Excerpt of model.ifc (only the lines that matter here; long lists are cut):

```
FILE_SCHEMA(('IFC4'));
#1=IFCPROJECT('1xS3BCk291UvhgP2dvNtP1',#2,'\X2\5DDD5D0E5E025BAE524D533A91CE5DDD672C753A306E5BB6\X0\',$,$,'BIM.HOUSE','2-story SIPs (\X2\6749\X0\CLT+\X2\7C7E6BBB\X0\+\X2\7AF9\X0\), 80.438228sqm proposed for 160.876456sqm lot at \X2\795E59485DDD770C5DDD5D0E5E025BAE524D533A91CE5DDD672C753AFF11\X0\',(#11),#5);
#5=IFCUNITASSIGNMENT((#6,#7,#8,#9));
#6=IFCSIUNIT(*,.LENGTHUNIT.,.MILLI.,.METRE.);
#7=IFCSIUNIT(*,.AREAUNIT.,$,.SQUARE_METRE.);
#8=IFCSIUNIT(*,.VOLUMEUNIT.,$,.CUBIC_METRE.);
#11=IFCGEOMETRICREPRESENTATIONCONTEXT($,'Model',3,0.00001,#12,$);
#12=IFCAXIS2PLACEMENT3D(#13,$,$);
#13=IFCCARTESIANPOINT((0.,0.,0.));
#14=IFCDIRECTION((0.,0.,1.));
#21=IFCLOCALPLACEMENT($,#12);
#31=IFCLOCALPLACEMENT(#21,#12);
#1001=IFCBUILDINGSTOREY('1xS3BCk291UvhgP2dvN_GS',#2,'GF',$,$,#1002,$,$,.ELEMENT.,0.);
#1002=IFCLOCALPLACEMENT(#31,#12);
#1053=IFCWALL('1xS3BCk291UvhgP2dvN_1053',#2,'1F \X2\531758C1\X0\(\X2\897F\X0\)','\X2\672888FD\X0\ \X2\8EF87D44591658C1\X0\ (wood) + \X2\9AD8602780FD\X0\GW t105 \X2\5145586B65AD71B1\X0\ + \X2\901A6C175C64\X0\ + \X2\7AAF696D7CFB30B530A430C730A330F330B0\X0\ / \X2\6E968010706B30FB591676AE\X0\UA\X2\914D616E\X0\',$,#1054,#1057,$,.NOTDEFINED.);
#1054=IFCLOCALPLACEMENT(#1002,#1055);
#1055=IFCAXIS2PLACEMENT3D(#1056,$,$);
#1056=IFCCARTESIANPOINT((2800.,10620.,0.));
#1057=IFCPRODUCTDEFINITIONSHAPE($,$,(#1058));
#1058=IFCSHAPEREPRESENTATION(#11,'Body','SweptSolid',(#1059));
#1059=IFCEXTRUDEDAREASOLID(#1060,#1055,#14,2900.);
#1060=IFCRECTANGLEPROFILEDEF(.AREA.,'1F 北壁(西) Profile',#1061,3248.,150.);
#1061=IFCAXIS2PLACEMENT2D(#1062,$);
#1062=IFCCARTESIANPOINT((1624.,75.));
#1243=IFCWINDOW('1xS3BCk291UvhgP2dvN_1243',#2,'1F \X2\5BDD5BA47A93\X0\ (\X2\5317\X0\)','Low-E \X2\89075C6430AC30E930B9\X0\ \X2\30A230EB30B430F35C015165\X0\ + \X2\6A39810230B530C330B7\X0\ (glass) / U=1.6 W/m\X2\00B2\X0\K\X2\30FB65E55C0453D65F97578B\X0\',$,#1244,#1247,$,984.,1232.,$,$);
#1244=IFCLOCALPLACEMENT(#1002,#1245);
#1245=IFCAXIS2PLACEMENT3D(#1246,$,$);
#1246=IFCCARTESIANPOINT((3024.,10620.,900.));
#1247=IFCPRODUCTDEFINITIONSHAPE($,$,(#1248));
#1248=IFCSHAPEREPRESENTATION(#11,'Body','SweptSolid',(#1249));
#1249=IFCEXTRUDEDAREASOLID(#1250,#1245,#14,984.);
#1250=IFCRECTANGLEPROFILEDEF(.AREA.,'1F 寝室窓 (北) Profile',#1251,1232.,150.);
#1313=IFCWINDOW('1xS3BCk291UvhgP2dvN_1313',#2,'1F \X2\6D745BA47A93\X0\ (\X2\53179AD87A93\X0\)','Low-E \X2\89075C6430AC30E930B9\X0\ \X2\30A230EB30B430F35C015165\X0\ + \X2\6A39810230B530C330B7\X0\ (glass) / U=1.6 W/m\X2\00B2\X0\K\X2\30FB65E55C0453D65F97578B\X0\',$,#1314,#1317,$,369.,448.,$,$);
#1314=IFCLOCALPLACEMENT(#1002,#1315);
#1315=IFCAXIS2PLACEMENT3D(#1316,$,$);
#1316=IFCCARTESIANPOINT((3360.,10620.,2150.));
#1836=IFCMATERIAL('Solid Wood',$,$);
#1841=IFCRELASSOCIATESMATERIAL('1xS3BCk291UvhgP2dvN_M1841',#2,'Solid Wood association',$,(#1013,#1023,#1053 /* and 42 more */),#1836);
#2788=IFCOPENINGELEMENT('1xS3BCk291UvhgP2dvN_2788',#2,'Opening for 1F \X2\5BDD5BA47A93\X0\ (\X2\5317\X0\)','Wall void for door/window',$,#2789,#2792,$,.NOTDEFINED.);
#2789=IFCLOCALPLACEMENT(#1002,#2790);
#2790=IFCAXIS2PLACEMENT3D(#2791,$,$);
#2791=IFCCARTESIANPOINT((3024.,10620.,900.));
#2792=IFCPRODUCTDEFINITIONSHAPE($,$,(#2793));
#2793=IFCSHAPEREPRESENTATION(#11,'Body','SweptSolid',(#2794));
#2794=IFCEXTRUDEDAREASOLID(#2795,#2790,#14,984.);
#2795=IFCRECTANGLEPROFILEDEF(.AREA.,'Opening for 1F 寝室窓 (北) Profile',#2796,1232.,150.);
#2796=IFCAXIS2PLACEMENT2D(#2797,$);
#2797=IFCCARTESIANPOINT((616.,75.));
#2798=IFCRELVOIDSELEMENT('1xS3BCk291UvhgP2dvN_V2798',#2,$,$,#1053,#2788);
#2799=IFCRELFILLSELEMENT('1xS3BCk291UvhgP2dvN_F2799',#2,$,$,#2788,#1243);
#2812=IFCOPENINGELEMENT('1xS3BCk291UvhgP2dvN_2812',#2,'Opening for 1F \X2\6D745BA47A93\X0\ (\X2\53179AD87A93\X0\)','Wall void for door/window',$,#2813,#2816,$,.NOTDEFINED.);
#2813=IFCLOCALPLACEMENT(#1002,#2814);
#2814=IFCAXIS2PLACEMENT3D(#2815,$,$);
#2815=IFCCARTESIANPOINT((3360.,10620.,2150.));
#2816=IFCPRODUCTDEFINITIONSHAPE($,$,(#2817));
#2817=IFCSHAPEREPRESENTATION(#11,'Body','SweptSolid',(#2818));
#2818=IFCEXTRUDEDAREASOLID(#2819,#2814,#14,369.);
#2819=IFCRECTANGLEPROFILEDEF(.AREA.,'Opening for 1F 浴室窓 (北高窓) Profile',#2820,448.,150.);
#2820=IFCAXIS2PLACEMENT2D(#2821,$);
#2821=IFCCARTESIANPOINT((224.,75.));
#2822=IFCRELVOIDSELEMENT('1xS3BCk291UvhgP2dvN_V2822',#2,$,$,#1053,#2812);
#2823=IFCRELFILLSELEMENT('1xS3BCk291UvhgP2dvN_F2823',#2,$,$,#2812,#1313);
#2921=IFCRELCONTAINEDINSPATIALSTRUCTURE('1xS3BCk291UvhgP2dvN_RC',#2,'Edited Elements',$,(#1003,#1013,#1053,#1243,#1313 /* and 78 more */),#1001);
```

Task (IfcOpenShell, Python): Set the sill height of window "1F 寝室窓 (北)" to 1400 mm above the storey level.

```python
import numpy as np
import ifcopenshell
import ifcopenshell.api.geometry
import ifcopenshell.geom
import ifcopenshell.util.element
import ifcopenshell.util.placement
import ifcopenshell.util.shape
import ifcopenshell.util.unit

model = ifcopenshell.open("model.ifc")
unit_scale = ifcopenshell.util.unit.calculate_unit_scale(model)

window = model.by_id(1243)
opening = window.FillsVoids[0].RelatingOpeningElement
storey = ifcopenshell.util.element.get_container(window, ifc_class="IfcBuildingStorey")
level = ifcopenshell.util.placement.get_local_placement(storey.ObjectPlacement)[2, 3]

# The opening's origin need not be at the sill, so measure its lowest point.
shape = ifcopenshell.geom.create_shape(ifcopenshell.geom.settings(), opening)
bottom = ifcopenshell.util.shape.get_shape_bottom_elevation(shape, shape.geometry) / unit_scale
dz = level + 1400.0 - bottom

shift = np.array([0.0, 0.0, dz])
# The window is not placed relative to its opening, so move both.
for product in (opening, window):
    matrix = ifcopenshell.util.placement.get_local_placement(product.ObjectPlacement)
    matrix[:3, 3] += shift
    ifcopenshell.api.geometry.edit_object_placement(model, product=product, matrix=matrix, is_si=False)

print(f"moved by {dz * unit_scale:+.3f} m")

model.write("model-out.ifc")
```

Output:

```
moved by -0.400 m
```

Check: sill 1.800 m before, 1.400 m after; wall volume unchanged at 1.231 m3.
